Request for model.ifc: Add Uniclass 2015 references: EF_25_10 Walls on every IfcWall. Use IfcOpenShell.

First a look at what the model holds.

```python
import ifcopenshell

model = ifcopenshell.open("model.ifc")
print(model.schema)
print("classifications:", [c.Name for c in model.by_type("IfcClassification")])
for ifc_class in ("IfcDoor", "IfcRoof", "IfcStair", "IfcWall", "IfcWindow"):
    print(ifc_class, len(model.by_type(ifc_class)))
```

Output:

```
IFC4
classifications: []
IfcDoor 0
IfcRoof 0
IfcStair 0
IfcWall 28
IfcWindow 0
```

```python
import ifcopenshell
import ifcopenshell.api.classification

model = ifcopenshell.open("model.ifc")

system = ifcopenshell.api.classification.add_classification(model, classification="Uniclass 2015")

codes = {
    "IfcWall": ("EF_25_10", "Walls"),
}
for ifc_class, (code, name) in codes.items():
    products = model.by_type(ifc_class)
    ifcopenshell.api.classification.add_reference(
        model, products=products, classification=system, identification=code, name=name
    )
    print(code, len(products))

model.write("model_updated.ifc")
```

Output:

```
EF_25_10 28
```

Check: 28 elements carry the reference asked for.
